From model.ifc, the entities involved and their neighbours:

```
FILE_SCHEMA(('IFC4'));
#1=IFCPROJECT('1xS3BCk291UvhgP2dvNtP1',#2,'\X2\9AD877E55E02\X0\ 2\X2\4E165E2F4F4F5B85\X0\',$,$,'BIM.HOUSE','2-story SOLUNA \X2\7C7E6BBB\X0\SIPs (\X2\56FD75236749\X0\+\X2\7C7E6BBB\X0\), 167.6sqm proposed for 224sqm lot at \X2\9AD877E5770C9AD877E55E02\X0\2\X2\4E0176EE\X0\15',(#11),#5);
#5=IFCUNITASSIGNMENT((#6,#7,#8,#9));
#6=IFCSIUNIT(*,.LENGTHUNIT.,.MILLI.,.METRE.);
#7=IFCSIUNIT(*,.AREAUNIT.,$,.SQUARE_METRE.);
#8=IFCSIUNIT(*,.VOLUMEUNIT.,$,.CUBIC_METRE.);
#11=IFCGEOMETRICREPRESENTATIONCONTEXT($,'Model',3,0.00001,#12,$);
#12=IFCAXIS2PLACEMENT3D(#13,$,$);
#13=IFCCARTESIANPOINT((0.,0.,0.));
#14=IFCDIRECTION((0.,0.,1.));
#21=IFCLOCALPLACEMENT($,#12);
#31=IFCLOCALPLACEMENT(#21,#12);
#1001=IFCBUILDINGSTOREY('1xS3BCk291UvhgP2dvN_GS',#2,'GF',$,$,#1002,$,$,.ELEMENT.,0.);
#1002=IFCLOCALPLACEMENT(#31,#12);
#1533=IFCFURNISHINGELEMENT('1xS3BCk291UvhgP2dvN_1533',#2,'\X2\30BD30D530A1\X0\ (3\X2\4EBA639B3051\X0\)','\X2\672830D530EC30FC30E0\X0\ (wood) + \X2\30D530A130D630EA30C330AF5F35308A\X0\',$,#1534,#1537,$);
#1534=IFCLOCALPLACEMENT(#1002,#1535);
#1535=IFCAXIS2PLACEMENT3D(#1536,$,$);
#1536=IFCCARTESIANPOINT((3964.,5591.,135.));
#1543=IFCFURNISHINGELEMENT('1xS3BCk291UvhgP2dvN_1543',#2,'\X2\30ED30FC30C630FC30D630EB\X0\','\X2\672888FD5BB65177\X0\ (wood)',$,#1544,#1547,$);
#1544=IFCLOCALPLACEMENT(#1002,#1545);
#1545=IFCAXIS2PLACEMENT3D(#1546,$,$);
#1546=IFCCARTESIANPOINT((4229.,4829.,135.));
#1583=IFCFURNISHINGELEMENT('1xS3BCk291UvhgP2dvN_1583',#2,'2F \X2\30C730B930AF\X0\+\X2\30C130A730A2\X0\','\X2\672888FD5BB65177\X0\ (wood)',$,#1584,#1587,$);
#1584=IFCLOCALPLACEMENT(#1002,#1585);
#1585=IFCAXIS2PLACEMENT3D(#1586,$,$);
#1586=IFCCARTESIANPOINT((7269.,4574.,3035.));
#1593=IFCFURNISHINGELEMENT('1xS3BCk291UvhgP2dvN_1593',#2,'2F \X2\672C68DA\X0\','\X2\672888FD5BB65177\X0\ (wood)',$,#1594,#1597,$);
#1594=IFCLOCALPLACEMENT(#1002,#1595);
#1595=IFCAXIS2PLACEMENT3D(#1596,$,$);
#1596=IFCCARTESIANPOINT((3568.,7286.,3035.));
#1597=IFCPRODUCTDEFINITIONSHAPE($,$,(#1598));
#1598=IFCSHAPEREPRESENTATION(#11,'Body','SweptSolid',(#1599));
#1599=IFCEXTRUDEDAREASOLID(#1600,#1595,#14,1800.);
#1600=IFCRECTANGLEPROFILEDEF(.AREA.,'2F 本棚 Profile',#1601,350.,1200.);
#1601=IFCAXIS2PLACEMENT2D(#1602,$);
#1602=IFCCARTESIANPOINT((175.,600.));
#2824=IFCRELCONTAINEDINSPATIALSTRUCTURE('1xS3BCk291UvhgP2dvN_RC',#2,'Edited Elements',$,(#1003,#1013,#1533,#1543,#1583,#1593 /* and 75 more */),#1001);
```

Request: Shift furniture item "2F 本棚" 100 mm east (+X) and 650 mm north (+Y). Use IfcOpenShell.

```python
import ifcopenshell
import ifcopenshell.api.geometry
import ifcopenshell.util.placement

model = ifcopenshell.open("model.ifc")

item = model.by_id(1593)
matrix = ifcopenshell.util.placement.get_local_placement(item.ObjectPlacement)
matrix[0, 3] += 100.0
matrix[1, 3] += 650.0
ifcopenshell.api.geometry.edit_object_placement(model, product=item, matrix=matrix, is_si=False)

print(ifcopenshell.util.placement.get_local_placement(item.ObjectPlacement).round(3) + 0.0)

model.write("model-out.ifc")
```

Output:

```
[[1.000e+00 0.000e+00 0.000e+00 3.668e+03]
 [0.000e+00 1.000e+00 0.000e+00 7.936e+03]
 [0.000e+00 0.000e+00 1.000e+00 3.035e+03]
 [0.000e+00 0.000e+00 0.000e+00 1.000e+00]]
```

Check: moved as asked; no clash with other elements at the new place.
